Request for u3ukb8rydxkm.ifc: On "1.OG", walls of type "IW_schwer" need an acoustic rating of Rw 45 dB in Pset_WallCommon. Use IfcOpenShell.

First a look at what the model holds.

```python
import ifcopenshell
import ifcopenshell.util.element

model = ifcopenshell.open("u3ukb8rydxkm.ifc")
print(model.schema)
storey = next(s for s in model.by_type("IfcBuildingStorey") if s.Name == "1.OG")
walls = [e for e in ifcopenshell.util.element.get_decomposition(storey) if e.is_a("IfcWall")]
seen = {}
for e in walls:
    element_type = ifcopenshell.util.element.get_type(e)
    key = (element_type.Name if element_type != e and element_type else None, ifcopenshell.util.element.get_pset(e, "Pset_WallCommon", "AcousticRating"))
    seen[key] = seen.get(key, 0) + 1
for (name, value), count in sorted(seen.items(), key=str):
    print(count, "x", name, "|", value)
```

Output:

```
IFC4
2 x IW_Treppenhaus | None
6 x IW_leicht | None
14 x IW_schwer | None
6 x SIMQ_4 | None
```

```python
import ifcopenshell
import ifcopenshell.api.pset
import ifcopenshell.util.element

model = ifcopenshell.open("u3ukb8rydxkm.ifc")

storey = next(s for s in model.by_type("IfcBuildingStorey") if s.Name == "1.OG")
walls = [e for e in ifcopenshell.util.element.get_decomposition(storey) if e.is_a("IfcWall")]

count = 0
for e in walls:
    element_type = ifcopenshell.util.element.get_type(e)
    if element_type in (None, e) or element_type.Name != "IW_schwer":
        continue
    # add_pset returns the element's existing set when there is one.
    pset = ifcopenshell.api.pset.add_pset(model, product=e, name="Pset_WallCommon")
    ifcopenshell.api.pset.edit_pset(model, pset=pset, properties={"AcousticRating": "Rw 45 dB"})
    count += 1

print(count, "walls updated")

model.write("u3ukb8rydxkm_v2.ifc")
```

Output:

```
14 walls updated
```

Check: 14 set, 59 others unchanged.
